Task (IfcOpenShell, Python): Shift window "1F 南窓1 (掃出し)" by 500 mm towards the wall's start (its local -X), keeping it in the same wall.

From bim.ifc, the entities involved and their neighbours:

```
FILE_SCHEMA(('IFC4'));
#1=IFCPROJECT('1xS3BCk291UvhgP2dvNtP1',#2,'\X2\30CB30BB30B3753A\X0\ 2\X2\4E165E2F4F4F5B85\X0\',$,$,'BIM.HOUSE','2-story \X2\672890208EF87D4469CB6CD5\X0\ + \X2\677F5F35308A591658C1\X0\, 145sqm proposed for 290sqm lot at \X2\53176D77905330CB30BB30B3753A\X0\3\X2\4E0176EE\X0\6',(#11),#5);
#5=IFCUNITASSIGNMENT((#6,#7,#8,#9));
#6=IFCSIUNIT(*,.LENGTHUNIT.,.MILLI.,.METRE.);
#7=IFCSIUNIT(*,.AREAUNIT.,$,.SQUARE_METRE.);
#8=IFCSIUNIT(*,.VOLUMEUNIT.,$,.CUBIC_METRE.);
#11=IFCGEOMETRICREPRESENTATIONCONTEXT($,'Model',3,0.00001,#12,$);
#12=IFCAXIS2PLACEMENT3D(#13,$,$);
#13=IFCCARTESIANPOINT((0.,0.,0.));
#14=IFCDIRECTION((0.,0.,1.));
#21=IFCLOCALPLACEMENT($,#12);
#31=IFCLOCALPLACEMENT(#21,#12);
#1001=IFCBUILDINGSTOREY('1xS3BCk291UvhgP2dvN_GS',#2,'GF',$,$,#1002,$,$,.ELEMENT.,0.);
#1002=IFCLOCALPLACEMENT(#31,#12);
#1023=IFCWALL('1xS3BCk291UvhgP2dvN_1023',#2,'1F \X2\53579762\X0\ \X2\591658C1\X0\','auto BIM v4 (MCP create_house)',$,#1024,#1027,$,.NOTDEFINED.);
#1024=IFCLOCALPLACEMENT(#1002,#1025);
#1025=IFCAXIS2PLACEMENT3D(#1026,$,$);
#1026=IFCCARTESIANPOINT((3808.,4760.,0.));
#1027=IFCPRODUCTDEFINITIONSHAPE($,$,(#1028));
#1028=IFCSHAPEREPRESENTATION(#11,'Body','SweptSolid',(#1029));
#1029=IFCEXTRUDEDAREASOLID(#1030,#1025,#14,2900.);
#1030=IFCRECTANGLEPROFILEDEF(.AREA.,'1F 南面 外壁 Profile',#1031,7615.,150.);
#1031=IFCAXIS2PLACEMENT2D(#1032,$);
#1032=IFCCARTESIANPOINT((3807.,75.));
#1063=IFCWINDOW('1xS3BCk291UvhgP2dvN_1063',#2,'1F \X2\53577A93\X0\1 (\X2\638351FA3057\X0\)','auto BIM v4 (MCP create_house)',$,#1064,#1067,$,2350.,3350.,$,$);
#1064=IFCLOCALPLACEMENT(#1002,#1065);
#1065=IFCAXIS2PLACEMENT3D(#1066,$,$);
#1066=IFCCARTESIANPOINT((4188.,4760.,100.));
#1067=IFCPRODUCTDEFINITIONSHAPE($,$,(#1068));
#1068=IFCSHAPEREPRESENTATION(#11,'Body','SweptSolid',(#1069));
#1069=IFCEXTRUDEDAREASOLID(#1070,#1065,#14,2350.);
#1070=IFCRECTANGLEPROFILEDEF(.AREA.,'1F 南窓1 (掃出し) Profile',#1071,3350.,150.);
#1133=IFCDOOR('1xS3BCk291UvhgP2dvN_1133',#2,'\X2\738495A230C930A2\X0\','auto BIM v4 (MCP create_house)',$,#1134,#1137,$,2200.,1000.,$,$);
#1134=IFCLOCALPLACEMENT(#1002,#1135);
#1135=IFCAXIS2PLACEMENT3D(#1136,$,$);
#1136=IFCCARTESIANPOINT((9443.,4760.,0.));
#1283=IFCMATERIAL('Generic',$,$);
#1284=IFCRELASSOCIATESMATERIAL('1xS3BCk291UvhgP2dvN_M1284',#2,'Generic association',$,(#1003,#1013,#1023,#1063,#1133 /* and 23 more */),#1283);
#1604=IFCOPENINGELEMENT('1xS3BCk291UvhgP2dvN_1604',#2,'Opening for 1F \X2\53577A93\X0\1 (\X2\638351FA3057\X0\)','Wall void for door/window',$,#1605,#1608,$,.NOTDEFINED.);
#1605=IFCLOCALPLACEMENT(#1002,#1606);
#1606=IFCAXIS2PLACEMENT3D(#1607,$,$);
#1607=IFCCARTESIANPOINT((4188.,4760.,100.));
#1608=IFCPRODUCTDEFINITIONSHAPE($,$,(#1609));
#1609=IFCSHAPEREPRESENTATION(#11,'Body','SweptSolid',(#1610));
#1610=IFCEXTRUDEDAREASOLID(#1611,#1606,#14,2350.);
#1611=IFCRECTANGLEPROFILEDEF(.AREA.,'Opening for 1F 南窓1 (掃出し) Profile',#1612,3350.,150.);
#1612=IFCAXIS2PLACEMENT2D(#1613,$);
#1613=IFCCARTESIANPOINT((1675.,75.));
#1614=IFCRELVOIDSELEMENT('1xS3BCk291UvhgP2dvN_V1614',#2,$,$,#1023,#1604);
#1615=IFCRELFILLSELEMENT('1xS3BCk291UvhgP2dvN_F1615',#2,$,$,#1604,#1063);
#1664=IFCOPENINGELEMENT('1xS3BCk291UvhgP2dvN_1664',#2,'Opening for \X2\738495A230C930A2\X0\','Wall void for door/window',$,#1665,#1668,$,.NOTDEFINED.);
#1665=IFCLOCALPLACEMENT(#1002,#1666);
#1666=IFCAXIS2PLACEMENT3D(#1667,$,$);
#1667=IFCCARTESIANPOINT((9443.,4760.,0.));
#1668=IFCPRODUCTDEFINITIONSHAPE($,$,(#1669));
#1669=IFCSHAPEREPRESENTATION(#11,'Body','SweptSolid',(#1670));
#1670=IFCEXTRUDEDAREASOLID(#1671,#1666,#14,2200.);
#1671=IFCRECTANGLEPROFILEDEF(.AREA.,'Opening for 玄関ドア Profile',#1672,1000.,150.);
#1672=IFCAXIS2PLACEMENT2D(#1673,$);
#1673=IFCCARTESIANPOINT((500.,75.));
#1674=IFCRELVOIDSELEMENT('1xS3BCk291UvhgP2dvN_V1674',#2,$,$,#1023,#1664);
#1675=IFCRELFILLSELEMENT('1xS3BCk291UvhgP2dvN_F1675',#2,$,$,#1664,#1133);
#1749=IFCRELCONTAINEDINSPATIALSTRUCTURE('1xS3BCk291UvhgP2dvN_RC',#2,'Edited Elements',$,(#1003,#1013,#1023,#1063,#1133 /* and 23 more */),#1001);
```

```python
import ifcopenshell
import ifcopenshell.api.geometry
import ifcopenshell.util.placement

model = ifcopenshell.open("bim.ifc")

window = model.by_id(1063)
opening = window.FillsVoids[0].RelatingOpeningElement
wall = opening.VoidsElements[0].RelatingBuildingElement

wall_matrix = ifcopenshell.util.placement.get_local_placement(wall.ObjectPlacement)
shift = wall_matrix[:3, 0] * -500.0
before = ifcopenshell.util.placement.get_local_placement(window.ObjectPlacement)[:3, 3].copy()

# The window is not placed relative to its opening, so move both.
for product in (opening, window):
    matrix = ifcopenshell.util.placement.get_local_placement(product.ObjectPlacement)
    matrix[:3, 3] += shift
    ifcopenshell.api.geometry.edit_object_placement(model, product=product, matrix=matrix, is_si=False)

after = ifcopenshell.util.placement.get_local_placement(window.ObjectPlacement)[:3, 3]
print("window moved by", (after - before).round(3) + 0.0)

model.write("bim_v2.ifc")
```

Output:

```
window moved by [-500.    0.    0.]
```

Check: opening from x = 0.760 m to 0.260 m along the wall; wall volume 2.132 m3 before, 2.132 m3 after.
